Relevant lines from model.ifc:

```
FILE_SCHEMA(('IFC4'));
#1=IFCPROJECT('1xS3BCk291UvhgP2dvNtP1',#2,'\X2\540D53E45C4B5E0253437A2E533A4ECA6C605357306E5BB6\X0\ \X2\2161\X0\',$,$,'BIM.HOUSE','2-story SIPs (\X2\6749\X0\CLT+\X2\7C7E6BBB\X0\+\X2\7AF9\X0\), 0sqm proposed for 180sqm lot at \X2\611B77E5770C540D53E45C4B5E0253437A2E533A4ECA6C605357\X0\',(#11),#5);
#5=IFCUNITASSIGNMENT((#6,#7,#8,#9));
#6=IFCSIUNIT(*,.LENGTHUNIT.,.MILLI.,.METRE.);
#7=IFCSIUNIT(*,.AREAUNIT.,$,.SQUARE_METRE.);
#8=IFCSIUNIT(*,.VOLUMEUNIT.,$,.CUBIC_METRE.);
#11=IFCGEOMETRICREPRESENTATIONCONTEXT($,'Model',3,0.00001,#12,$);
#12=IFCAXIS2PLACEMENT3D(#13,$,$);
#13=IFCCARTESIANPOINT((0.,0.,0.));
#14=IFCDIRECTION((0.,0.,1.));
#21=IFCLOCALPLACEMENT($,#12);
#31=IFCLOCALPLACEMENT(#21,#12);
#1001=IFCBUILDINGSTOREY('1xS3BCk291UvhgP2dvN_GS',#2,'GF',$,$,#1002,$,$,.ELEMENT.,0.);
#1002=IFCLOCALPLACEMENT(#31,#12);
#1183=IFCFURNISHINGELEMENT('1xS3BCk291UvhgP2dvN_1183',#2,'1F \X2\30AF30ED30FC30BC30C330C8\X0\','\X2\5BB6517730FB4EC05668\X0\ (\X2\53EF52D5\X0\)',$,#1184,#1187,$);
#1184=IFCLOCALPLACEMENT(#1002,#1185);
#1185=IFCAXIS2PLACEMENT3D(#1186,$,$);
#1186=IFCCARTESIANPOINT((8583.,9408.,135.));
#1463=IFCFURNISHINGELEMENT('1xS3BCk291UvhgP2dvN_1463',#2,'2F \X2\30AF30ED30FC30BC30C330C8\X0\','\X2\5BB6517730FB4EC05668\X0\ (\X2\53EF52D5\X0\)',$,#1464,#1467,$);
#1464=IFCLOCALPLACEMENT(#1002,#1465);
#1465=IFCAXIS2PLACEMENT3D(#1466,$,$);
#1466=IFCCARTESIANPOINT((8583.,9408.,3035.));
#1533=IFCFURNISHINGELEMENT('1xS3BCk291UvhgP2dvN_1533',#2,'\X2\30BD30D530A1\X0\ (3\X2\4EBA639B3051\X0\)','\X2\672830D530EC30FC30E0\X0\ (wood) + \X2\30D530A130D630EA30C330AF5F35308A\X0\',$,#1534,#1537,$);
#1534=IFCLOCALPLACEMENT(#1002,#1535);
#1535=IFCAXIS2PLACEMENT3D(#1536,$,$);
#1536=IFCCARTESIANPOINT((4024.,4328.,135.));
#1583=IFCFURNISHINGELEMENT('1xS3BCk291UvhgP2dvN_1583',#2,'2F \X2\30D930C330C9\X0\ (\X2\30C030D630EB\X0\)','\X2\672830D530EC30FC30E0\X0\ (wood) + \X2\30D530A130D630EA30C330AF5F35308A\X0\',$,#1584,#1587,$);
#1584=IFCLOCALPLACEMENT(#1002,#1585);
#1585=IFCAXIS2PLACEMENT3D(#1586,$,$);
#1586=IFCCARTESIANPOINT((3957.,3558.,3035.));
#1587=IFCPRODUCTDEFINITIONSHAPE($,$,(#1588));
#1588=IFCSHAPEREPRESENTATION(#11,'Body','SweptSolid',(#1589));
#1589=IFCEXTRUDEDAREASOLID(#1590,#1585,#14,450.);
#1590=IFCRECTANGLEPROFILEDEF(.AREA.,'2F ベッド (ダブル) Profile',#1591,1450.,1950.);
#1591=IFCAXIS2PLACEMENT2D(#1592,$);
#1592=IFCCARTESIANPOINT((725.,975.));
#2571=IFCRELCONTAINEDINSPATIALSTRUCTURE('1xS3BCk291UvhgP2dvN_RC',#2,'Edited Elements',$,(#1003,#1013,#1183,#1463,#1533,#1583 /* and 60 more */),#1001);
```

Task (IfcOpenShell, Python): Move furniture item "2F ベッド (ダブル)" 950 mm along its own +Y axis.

```python
import ifcopenshell
import ifcopenshell.api.geometry
import ifcopenshell.util.placement

model = ifcopenshell.open("model.ifc")

item = model.by_guid("1xS3BCk291UvhgP2dvN_1583")
matrix = ifcopenshell.util.placement.get_local_placement(item.ObjectPlacement)
matrix[:3, 3] += matrix[:3, 1] * 950.0
ifcopenshell.api.geometry.edit_object_placement(model, product=item, matrix=matrix, is_si=False)

print(ifcopenshell.util.placement.get_local_placement(item.ObjectPlacement).round(3) + 0.0)

model.write("model_rev.ifc")
```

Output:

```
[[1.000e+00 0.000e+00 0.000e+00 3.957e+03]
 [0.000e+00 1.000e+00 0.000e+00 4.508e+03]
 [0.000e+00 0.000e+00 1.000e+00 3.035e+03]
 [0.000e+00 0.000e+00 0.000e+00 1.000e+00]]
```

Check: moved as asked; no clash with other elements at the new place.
